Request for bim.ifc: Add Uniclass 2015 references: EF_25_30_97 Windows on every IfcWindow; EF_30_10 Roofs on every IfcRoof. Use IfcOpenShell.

First a look at what the model holds.

```python
import ifcopenshell

model = ifcopenshell.open("bim.ifc")
print(model.schema)
print("classifications:", [c.Name for c in model.by_type("IfcClassification")])
for ifc_class in ("IfcDoor", "IfcRoof", "IfcStair", "IfcWall", "IfcWindow"):
    print(ifc_class, len(model.by_type(ifc_class)))
```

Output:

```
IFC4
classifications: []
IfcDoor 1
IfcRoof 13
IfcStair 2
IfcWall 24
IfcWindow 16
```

```python
import ifcopenshell
import ifcopenshell.api.classification

model = ifcopenshell.open("bim.ifc")

system = ifcopenshell.api.classification.add_classification(model, classification="Uniclass 2015")

codes = {
    "IfcWindow": ("EF_25_30_97", "Windows"),
    "IfcRoof": ("EF_30_10", "Roofs"),
}
for ifc_class, (code, name) in codes.items():
    products = model.by_type(ifc_class)
    ifcopenshell.api.classification.add_reference(
        model, products=products, classification=system, identification=code, name=name
    )
    print(code, len(products))

model.write("bim_updated.ifc")
```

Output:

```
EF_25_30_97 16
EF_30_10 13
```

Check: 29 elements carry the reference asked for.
